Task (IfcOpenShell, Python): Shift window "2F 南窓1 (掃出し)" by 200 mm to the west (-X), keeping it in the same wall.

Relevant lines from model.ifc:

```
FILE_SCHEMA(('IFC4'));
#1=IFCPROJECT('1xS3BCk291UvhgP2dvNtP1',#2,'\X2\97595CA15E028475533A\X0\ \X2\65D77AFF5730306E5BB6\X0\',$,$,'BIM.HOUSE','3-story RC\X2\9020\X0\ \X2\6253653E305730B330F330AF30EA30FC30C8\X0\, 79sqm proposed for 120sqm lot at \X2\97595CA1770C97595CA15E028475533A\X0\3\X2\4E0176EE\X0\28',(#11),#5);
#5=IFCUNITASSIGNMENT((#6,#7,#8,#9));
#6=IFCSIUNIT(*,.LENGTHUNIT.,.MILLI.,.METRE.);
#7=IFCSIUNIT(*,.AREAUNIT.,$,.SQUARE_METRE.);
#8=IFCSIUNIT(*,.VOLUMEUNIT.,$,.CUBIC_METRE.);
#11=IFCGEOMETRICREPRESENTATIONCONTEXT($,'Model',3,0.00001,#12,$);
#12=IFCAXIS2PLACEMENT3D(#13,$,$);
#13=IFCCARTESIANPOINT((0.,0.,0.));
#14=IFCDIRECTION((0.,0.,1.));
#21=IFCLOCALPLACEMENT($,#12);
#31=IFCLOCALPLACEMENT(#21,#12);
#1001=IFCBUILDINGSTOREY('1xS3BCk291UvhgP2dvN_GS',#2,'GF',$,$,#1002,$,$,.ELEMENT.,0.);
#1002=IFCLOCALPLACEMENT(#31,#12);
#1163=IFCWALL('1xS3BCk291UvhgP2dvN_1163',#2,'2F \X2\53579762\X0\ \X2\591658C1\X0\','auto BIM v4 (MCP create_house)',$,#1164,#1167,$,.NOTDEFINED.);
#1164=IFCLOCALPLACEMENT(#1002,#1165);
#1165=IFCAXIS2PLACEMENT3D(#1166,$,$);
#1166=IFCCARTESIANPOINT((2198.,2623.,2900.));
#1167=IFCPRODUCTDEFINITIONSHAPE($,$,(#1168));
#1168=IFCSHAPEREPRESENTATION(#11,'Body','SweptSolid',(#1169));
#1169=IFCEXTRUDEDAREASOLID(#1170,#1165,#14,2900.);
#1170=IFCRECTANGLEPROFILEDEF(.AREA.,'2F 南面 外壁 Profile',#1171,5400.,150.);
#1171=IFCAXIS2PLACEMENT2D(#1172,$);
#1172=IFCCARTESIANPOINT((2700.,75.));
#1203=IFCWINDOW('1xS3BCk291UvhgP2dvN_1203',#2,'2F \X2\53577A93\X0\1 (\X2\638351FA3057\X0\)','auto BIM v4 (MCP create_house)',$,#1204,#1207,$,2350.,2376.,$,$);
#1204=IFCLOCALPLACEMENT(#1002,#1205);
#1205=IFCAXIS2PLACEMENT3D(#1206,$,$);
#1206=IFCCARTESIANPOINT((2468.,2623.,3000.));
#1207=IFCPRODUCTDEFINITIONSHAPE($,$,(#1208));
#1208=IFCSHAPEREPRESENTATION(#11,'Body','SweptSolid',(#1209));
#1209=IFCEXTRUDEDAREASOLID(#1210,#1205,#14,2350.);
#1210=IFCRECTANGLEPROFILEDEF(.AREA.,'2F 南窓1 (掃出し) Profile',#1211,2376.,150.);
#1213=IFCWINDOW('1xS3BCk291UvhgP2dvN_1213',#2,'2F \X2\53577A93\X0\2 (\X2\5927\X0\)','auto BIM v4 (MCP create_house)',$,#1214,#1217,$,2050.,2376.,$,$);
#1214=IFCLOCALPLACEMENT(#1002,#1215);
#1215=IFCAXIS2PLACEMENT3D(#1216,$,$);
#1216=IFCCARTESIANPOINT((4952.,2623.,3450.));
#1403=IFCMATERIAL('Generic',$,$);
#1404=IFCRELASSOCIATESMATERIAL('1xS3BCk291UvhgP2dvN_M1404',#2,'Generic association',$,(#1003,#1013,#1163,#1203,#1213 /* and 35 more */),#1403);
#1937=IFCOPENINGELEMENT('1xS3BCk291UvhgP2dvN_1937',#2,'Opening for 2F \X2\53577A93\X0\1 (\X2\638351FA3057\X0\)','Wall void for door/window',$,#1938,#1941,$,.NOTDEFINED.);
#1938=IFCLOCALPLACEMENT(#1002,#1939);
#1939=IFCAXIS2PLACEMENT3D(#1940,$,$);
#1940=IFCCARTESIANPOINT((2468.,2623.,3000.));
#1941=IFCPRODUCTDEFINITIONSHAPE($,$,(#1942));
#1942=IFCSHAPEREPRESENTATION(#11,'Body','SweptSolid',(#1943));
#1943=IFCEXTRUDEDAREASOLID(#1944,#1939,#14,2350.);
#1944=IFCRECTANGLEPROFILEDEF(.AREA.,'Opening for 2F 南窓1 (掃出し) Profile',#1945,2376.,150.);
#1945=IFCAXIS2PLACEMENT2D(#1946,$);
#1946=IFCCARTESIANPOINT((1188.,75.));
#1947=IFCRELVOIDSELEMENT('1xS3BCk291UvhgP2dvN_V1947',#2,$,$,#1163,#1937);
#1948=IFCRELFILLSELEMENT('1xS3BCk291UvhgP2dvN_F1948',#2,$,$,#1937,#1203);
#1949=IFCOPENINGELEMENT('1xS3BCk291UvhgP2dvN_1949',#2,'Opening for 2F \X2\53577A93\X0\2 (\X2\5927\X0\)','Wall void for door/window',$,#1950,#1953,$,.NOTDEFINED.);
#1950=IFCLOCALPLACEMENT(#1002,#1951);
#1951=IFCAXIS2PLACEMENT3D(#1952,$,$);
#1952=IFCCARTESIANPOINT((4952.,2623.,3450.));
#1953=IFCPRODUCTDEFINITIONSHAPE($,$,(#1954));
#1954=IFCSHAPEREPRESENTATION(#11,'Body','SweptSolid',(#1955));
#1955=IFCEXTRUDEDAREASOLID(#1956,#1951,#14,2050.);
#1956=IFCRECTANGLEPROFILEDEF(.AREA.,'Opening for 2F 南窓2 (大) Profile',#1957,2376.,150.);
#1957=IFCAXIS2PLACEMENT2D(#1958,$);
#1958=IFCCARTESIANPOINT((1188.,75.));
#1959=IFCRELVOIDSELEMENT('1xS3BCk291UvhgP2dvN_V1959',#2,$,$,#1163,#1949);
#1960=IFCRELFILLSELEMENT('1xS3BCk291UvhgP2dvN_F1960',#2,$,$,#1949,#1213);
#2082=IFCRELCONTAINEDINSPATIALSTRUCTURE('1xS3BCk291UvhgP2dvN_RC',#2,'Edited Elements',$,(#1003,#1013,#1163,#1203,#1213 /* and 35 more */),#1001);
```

```python
import ifcopenshell
import ifcopenshell.api.geometry
import ifcopenshell.util.placement
import ifcopenshell.util.unit

model = ifcopenshell.open("model.ifc")
unit_scale = ifcopenshell.util.unit.calculate_unit_scale(model)

window = model.by_guid("1xS3BCk291UvhgP2dvN_1203")
opening = window.FillsVoids[0].RelatingOpeningElement
wall = opening.VoidsElements[0].RelatingBuildingElement

wall_matrix = ifcopenshell.util.placement.get_local_placement(wall.ObjectPlacement)
shift = wall_matrix[:3, 0] * -0.2 / unit_scale
before = ifcopenshell.util.placement.get_local_placement(window.ObjectPlacement)[:3, 3].copy()

# The window is not placed relative to its opening, so move both.
for product in (opening, window):
    matrix = ifcopenshell.util.placement.get_local_placement(product.ObjectPlacement)
    matrix[:3, 3] += shift
    ifcopenshell.api.geometry.edit_object_placement(model, product=product, matrix=matrix, is_si=False)

after = ifcopenshell.util.placement.get_local_placement(window.ObjectPlacement)[:3, 3]
print("window moved by", (after - before).round(3) + 0.0)

model.write("model-out.ifc")
```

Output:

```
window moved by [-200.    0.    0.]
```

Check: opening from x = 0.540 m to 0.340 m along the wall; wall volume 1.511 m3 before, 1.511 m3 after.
